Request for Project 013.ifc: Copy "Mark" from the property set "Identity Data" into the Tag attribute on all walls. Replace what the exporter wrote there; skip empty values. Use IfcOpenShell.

First a look at what the model holds.

```python
import ifcopenshell
import ifcopenshell.util.element

model = ifcopenshell.open("Project 013.ifc")
print(model.schema)
walls = model.by_type("IfcWall")
print(len(walls), "walls")
for e in walls[:8]:
    source = ifcopenshell.util.element.get_pset(e, "Identity Data", "Mark")
    target = e.Tag
    print(e.id(), repr(source), repr(target), sep=" | ")
```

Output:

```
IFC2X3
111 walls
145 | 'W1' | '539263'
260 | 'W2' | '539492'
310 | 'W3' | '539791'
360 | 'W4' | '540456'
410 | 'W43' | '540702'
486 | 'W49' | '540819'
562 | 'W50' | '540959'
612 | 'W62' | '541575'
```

```python
import ifcopenshell
import ifcopenshell.util.element

model = ifcopenshell.open("Project 013.ifc")

count = 0
for e in model.by_type("IfcWall"):
    value = ifcopenshell.util.element.get_pset(e, "Identity Data", "Mark")
    current = e.Tag
    if not value or not value.strip() or current == value:
        continue
    e.Tag = value
    count += 1

print(count, "walls updated")

model.write("Project 013_v2.ifc")
```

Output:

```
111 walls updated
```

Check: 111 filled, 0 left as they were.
